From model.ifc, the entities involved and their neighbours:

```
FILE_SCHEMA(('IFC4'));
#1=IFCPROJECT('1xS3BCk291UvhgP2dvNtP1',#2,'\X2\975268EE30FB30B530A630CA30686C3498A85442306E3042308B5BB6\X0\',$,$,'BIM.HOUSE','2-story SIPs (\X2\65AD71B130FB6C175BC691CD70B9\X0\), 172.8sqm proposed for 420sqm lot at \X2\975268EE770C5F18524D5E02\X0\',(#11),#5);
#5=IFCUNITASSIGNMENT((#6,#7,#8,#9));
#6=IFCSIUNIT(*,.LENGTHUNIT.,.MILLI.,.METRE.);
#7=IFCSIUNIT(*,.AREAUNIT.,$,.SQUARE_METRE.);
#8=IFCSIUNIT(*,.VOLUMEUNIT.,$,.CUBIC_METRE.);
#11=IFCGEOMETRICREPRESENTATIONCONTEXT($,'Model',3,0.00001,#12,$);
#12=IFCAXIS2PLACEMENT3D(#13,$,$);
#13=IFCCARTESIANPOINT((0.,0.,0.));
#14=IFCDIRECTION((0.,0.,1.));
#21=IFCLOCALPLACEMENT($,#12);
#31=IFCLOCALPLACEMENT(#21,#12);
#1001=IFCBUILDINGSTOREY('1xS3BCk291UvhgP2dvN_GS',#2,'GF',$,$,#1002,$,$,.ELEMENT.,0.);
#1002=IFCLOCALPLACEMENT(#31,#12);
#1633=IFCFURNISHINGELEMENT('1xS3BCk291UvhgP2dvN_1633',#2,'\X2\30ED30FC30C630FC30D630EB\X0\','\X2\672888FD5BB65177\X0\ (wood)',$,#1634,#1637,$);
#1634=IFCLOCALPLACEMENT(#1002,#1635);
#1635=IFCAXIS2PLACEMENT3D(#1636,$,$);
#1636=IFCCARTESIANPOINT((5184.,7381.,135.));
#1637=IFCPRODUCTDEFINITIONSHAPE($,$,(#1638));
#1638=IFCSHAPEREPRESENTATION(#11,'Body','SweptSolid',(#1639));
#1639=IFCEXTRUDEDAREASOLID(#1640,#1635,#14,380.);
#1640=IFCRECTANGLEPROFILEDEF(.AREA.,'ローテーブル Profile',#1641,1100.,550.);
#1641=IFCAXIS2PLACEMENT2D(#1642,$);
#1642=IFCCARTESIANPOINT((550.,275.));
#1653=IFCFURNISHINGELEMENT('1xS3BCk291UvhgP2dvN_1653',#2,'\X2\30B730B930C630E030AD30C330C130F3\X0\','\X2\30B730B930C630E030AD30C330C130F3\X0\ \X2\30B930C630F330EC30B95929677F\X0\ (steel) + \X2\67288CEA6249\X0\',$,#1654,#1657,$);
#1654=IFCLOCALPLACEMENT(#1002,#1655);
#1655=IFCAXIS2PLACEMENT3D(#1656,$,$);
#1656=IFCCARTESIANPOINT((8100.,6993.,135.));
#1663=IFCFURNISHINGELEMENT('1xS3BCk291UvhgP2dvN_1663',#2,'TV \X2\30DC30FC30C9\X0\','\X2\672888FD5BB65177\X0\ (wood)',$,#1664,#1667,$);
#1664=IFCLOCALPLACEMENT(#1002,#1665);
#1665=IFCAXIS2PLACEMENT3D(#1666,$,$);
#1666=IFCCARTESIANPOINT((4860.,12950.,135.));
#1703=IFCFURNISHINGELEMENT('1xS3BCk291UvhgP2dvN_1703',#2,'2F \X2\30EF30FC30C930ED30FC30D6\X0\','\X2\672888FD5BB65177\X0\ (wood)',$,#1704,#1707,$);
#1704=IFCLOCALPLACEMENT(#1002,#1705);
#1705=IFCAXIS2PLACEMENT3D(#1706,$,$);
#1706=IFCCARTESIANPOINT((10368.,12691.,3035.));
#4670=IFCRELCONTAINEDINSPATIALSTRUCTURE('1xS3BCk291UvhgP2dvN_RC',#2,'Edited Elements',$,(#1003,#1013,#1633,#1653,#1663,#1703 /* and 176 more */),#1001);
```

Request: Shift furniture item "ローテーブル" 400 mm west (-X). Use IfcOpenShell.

```python
import ifcopenshell
import ifcopenshell.api.geometry
import ifcopenshell.util.placement

model = ifcopenshell.open("model.ifc")

item = model.by_guid("1xS3BCk291UvhgP2dvN_1633")
matrix = ifcopenshell.util.placement.get_local_placement(item.ObjectPlacement)
matrix[0, 3] -= 400.0
ifcopenshell.api.geometry.edit_object_placement(model, product=item, matrix=matrix, is_si=False)

print(ifcopenshell.util.placement.get_local_placement(item.ObjectPlacement).round(3) + 0.0)

model.write("model_rev.ifc")
```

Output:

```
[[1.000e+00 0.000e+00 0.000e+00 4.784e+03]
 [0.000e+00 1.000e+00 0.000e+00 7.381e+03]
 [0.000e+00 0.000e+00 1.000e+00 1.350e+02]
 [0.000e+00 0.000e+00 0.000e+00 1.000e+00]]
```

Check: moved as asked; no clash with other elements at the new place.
